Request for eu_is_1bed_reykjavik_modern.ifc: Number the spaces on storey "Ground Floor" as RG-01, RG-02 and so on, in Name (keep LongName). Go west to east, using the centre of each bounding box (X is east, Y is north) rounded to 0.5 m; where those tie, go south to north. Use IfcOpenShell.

First a look at what the model holds.

```python
import ifcopenshell
import ifcopenshell.util.element
import ifcopenshell.util.placement

model = ifcopenshell.open("eu_is_1bed_reykjavik_modern.ifc")
print(model.schema)
storey = next(s for s in model.by_type("IfcBuildingStorey") if s.Name == "Ground Floor")
spaces = [e for e in ifcopenshell.util.element.get_decomposition(storey) if e.is_a("IfcSpace")]
for e in sorted(spaces, key=lambda e: e.id()):
    origin = ifcopenshell.util.placement.get_local_placement(e.ObjectPlacement)[:3, 3]
    print(e.id(), e.Name, e.LongName, origin.round(2) + 0.0, sep=" | ")
```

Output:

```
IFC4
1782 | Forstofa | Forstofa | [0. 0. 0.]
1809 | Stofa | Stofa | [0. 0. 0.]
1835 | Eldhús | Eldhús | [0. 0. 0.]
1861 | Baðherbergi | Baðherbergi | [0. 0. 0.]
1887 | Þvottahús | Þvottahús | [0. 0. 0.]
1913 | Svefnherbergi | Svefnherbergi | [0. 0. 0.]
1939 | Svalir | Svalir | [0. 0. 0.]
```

```python
import ifcopenshell
import ifcopenshell.geom
import ifcopenshell.util.element
import ifcopenshell.util.shape

model = ifcopenshell.open("eu_is_1bed_reykjavik_modern.ifc")
settings = ifcopenshell.geom.settings()
settings.set("use-world-coords", True)


def centre(element):
    shape = ifcopenshell.geom.create_shape(settings, element)
    return ifcopenshell.util.shape.get_bbox_centroid(shape.geometry)


storey = next(s for s in model.by_type("IfcBuildingStorey") if s.Name == "Ground Floor")
spaces = [e for e in ifcopenshell.util.element.get_decomposition(storey) if e.is_a("IfcSpace")]

# Insertion points can sit at a corner or the storey origin, so sort by the geometry (in metres).
centres = {e: centre(e) for e in spaces}
spaces.sort(key=lambda e: (round(centres[e][0] / 0.5), centres[e][1]))

for i, e in enumerate(spaces, start=1):
    number = f"RG-{i:02d}"
    e.Name = number
    print(e.id(), number)

model.write("eu_is_1bed_reykjavik_modern_v2.ifc")
```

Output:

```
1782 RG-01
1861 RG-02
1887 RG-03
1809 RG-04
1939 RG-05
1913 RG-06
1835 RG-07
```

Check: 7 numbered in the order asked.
